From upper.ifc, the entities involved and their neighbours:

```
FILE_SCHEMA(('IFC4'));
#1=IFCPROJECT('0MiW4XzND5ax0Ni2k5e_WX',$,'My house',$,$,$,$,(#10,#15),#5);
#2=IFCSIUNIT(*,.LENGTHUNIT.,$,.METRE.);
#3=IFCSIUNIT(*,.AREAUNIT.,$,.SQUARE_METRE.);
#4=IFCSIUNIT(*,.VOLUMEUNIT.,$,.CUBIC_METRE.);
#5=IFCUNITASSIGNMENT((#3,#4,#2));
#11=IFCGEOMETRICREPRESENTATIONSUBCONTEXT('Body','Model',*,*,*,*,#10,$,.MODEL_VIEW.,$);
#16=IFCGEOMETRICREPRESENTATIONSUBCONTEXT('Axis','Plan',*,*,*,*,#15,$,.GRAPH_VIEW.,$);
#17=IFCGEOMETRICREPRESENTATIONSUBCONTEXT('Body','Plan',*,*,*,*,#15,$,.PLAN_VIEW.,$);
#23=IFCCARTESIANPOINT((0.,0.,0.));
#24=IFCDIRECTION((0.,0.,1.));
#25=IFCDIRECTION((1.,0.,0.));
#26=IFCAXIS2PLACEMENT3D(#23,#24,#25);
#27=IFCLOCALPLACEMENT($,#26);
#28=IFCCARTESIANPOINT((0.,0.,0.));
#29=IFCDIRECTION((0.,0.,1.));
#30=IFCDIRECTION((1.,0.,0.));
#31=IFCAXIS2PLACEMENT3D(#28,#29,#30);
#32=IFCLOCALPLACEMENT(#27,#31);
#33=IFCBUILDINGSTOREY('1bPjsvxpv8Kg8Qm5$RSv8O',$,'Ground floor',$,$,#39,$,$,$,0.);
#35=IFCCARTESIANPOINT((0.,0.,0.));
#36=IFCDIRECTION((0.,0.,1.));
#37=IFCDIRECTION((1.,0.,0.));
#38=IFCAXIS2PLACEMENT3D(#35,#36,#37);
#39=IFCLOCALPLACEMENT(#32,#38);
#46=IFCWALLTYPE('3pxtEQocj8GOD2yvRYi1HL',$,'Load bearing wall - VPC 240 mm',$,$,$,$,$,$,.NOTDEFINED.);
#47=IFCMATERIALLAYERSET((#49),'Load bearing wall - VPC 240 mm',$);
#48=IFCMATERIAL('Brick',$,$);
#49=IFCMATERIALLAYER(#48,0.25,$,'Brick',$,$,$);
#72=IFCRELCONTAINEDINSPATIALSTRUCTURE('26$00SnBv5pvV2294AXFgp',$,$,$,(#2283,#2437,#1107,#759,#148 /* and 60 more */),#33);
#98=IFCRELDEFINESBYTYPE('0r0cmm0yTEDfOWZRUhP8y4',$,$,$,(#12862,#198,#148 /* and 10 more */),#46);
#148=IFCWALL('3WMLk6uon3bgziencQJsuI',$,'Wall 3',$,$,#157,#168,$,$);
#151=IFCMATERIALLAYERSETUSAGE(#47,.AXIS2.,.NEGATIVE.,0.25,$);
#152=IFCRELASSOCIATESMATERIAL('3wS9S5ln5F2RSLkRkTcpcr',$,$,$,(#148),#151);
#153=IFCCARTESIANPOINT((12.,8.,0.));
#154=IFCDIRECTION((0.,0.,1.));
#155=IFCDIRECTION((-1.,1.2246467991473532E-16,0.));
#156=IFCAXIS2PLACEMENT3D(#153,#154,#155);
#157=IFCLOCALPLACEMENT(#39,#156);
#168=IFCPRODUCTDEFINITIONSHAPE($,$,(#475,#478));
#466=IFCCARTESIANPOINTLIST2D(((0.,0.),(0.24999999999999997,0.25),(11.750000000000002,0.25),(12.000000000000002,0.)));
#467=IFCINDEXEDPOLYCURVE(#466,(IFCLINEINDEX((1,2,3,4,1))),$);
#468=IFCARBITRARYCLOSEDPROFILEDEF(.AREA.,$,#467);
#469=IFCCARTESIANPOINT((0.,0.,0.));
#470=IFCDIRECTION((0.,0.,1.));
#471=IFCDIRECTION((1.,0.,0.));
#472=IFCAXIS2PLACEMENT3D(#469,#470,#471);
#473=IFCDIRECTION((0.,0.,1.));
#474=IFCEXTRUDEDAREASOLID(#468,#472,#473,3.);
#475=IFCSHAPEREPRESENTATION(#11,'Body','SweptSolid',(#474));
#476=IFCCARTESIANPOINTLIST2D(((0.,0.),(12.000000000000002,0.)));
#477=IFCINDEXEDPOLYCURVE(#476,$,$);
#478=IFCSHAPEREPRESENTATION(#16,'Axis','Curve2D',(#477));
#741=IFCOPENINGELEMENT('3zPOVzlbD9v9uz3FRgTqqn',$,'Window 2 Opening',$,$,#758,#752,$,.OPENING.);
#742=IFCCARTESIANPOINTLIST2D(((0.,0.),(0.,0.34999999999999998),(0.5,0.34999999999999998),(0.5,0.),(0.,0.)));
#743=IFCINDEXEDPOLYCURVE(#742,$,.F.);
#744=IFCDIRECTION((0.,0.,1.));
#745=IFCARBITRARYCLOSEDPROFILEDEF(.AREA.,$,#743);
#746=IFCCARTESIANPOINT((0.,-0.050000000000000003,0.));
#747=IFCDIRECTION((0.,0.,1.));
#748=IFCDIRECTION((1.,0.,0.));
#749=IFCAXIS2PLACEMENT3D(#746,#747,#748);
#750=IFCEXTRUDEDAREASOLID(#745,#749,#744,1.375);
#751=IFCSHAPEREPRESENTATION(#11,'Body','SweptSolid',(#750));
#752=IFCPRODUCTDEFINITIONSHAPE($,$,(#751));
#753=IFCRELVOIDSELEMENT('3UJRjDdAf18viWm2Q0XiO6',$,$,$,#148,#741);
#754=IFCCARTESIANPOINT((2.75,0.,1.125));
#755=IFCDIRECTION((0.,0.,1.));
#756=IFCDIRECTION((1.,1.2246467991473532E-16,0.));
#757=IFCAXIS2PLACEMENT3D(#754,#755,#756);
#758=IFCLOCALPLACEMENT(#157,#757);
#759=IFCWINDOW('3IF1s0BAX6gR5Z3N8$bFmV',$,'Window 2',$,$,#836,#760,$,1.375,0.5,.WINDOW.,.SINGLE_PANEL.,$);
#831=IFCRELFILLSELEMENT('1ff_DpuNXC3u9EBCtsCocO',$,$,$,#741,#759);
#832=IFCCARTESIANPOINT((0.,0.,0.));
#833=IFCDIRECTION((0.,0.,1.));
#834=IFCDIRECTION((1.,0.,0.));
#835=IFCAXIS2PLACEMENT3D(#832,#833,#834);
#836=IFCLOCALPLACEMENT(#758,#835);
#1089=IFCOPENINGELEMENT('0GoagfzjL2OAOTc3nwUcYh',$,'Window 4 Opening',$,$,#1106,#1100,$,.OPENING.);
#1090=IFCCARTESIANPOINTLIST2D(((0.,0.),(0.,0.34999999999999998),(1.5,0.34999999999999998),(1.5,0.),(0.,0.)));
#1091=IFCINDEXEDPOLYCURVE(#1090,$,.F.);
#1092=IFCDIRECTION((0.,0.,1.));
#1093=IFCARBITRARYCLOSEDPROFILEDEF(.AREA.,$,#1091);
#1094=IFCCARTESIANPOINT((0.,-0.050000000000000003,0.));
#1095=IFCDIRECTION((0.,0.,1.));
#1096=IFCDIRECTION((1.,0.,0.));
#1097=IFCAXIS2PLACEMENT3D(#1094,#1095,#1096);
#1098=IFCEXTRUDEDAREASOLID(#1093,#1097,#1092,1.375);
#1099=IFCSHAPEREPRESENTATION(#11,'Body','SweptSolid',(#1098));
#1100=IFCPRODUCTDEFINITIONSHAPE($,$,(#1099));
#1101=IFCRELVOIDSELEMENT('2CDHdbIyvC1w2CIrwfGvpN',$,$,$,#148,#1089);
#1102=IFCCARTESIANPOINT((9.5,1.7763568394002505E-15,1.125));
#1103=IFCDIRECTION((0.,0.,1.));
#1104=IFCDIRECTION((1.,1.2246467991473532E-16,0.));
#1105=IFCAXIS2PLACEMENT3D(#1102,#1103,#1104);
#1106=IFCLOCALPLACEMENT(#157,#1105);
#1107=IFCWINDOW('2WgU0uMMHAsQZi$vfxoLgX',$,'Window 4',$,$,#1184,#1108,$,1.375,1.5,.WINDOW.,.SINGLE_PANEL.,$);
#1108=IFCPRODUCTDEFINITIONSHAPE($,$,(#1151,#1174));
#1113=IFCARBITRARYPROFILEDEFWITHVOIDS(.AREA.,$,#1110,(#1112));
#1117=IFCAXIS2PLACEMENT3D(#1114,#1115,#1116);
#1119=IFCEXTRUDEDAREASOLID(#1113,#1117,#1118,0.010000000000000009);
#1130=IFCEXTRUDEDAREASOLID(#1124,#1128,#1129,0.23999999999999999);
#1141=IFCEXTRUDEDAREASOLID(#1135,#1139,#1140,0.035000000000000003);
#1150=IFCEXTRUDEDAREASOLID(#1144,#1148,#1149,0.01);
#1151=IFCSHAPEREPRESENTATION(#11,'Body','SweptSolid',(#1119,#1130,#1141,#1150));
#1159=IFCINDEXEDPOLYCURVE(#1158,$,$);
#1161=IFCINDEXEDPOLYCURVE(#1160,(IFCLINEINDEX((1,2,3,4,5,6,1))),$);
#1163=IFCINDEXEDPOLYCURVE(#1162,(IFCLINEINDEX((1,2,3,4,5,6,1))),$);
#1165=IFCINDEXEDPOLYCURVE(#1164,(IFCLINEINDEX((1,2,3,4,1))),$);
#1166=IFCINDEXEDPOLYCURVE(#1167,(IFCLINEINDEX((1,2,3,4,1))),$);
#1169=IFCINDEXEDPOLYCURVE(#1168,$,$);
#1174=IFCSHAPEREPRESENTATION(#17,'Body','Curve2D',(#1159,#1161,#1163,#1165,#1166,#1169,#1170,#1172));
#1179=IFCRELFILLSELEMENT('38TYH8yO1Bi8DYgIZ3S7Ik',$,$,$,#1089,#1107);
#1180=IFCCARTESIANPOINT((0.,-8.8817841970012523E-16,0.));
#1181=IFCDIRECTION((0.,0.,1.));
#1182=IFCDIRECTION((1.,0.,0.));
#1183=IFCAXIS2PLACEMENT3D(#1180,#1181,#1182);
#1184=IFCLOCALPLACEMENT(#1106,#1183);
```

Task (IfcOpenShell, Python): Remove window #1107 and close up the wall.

```python
import ifcopenshell
import ifcopenshell.api.feature
import ifcopenshell.api.root
import ifcopenshell.geom
import ifcopenshell.util.shape

model = ifcopenshell.open("upper.ifc")
settings = ifcopenshell.geom.settings()


def volume(element):
    """Net volume in cubic metres, openings subtracted."""
    shape = ifcopenshell.geom.create_shape(settings, element)
    return ifcopenshell.util.shape.get_volume(shape.geometry)


window = model.by_id(1107)
opening = window.FillsVoids[0].RelatingOpeningElement
wall = opening.VoidsElements[0].RelatingBuildingElement
before = volume(wall)

ifcopenshell.api.root.remove_product(model, product=window)
ifcopenshell.api.feature.remove_feature(model, feature=opening)

after = volume(wall)

print(f"wall volume {before:.3f} -> {after:.3f} m3")

model.write("upper_rev.ifc")
```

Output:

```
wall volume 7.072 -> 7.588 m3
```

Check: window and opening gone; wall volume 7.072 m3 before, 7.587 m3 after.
